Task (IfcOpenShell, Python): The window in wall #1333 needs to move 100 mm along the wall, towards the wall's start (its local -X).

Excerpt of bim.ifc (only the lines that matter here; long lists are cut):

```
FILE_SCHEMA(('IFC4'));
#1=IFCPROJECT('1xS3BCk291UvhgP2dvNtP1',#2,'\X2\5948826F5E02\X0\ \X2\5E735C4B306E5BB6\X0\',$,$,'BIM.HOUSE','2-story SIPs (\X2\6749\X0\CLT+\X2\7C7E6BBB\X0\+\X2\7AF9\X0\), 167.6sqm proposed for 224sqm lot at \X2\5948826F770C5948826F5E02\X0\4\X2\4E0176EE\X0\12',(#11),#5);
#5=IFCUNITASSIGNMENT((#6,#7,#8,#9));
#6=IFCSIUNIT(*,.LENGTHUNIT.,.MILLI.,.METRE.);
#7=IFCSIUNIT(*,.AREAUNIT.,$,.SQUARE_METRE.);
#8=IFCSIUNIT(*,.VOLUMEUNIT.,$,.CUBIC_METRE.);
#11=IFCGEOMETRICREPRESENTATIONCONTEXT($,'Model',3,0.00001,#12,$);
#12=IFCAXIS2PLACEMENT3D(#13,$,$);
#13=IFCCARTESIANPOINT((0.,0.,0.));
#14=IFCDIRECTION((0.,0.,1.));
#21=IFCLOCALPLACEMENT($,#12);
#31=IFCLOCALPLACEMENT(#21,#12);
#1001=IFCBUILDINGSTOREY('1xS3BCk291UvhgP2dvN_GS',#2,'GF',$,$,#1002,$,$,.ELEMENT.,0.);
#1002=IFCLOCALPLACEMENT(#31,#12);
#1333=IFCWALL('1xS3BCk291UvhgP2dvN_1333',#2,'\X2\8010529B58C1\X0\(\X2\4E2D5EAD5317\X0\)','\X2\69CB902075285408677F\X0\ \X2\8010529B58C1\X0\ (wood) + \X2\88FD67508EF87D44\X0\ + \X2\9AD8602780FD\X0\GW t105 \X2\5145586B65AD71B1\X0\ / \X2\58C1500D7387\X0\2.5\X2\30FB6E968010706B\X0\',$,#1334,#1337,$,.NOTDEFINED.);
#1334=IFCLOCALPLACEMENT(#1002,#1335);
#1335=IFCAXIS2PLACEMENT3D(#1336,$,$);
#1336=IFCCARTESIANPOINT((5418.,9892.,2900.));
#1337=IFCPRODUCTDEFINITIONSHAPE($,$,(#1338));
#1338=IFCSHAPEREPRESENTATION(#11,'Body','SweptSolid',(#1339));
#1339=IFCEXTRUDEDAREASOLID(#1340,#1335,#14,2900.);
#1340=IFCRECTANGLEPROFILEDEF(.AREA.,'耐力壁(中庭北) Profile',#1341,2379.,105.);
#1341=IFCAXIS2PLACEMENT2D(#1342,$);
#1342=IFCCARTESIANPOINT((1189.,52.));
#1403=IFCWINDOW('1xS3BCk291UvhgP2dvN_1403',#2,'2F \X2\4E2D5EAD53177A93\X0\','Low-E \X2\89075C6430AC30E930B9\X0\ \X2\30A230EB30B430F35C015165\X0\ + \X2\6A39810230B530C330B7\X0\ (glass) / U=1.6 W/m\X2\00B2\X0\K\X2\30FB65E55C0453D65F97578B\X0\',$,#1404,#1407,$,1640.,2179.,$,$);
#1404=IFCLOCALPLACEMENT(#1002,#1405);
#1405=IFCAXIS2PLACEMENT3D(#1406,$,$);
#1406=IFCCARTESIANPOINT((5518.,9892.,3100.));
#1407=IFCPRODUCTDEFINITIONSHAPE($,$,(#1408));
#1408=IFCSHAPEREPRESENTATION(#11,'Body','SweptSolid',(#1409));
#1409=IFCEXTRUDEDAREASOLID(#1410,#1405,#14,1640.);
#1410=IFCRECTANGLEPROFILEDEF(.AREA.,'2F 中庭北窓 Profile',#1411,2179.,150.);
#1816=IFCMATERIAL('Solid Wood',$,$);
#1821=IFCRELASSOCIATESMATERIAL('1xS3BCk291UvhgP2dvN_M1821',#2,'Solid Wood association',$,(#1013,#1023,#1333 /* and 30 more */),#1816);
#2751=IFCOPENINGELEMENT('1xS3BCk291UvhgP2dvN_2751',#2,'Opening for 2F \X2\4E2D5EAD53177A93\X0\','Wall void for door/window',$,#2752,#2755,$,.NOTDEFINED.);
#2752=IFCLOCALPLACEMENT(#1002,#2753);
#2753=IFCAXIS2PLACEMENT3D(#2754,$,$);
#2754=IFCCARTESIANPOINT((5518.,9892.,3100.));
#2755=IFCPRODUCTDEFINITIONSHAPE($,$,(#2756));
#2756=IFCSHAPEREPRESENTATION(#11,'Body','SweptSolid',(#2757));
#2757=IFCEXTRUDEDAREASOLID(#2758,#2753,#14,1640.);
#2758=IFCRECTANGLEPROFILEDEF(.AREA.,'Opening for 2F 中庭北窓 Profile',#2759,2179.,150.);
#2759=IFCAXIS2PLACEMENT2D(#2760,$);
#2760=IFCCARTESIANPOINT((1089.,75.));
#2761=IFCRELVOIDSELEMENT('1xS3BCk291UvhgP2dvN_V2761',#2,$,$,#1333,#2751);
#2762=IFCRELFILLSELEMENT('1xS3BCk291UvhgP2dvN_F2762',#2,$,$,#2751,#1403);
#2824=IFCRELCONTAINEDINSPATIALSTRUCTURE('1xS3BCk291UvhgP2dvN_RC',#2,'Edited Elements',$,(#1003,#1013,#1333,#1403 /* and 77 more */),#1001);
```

```python
import ifcopenshell
import ifcopenshell.api.geometry
import ifcopenshell.util.placement

model = ifcopenshell.open("bim.ifc")

window = model.by_guid("1xS3BCk291UvhgP2dvN_1403")
opening = window.FillsVoids[0].RelatingOpeningElement
wall = opening.VoidsElements[0].RelatingBuildingElement

wall_matrix = ifcopenshell.util.placement.get_local_placement(wall.ObjectPlacement)
shift = wall_matrix[:3, 0] * -100.0
before = ifcopenshell.util.placement.get_local_placement(window.ObjectPlacement)[:3, 3].copy()

# The window is not placed relative to its opening, so move both.
for product in (opening, window):
    matrix = ifcopenshell.util.placement.get_local_placement(product.ObjectPlacement)
    matrix[:3, 3] += shift
    ifcopenshell.api.geometry.edit_object_placement(model, product=product, matrix=matrix, is_si=False)

after = ifcopenshell.util.placement.get_local_placement(window.ObjectPlacement)[:3, 3]
print("window moved by", (after - before).round(3) + 0.0)

model.write("bim_edited.ifc")
```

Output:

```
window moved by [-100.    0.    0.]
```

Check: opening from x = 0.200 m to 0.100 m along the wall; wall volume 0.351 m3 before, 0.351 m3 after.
